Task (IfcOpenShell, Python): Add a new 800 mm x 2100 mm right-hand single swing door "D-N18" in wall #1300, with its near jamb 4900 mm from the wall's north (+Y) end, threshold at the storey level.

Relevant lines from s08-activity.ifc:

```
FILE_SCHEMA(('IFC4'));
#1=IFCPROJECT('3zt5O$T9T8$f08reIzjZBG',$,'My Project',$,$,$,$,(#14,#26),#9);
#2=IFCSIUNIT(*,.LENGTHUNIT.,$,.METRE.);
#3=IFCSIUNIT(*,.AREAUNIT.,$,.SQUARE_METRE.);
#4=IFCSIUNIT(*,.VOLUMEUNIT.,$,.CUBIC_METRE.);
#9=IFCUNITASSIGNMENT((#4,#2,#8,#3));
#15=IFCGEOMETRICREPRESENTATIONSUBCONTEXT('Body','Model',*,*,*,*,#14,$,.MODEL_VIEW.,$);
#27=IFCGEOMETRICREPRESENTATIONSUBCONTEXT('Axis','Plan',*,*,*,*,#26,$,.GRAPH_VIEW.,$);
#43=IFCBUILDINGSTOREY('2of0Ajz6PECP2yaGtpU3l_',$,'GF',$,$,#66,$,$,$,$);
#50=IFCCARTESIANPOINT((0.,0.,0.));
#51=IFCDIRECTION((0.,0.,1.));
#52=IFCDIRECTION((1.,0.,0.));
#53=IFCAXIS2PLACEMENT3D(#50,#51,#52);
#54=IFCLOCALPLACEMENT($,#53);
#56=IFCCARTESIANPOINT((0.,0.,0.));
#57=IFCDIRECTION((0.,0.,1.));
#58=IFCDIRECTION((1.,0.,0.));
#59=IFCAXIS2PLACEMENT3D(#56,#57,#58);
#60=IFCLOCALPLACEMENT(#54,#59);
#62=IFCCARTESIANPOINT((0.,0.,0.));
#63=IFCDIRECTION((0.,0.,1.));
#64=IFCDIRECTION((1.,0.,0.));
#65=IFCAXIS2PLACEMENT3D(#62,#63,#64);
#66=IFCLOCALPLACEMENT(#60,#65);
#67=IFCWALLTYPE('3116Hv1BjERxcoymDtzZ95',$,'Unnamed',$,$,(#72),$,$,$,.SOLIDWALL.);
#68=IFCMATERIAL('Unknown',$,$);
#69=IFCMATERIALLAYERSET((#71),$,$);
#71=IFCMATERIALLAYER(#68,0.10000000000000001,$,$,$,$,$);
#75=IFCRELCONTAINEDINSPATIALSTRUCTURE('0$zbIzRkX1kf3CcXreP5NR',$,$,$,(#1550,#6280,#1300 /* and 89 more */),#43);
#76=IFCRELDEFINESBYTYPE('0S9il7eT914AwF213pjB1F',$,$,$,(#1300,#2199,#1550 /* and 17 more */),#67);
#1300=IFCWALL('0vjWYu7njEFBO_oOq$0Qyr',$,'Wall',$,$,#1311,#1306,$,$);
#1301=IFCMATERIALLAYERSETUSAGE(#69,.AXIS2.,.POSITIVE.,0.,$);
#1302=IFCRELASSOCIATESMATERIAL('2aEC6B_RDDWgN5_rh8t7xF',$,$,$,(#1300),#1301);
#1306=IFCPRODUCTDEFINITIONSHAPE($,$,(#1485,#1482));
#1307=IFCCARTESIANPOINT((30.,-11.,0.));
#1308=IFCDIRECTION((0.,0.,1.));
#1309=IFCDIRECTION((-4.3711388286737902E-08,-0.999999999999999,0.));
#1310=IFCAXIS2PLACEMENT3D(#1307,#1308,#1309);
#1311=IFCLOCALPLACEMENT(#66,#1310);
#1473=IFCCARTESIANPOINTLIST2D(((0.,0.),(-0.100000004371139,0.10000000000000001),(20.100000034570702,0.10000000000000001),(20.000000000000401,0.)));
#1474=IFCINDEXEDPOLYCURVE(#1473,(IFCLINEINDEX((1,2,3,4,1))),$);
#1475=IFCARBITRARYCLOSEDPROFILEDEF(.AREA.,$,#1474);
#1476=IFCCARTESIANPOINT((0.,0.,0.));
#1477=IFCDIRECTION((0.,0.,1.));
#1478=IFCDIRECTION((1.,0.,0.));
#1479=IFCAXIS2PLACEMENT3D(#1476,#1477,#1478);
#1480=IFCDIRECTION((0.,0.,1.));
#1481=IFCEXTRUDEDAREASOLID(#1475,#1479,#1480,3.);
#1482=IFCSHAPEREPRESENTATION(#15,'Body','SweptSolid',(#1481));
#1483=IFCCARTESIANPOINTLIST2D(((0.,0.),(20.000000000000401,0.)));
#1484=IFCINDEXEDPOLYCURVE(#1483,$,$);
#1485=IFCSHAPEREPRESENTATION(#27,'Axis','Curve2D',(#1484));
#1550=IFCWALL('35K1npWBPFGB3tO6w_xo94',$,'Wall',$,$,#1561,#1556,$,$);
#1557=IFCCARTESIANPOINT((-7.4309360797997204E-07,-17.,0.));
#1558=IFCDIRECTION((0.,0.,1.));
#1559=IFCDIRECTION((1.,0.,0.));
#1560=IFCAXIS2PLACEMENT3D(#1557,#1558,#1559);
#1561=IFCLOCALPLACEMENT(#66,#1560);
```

```python
import numpy as np
import ifcopenshell
import ifcopenshell.api.feature
import ifcopenshell.api.geometry
import ifcopenshell.api.root
import ifcopenshell.api.spatial
import ifcopenshell.geom
import ifcopenshell.util.element
import ifcopenshell.util.placement
import ifcopenshell.util.representation
import ifcopenshell.util.shape
import ifcopenshell.util.unit

model = ifcopenshell.open("s08-activity.ifc")
unit_scale = ifcopenshell.util.unit.calculate_unit_scale(model)
settings = ifcopenshell.geom.settings()


def volume(element):
    """Net volume in cubic metres, openings subtracted."""
    shape = ifcopenshell.geom.create_shape(settings, element)
    return ifcopenshell.util.shape.get_volume(shape.geometry)


wall = model.by_guid("0vjWYu7njEFBO_oOq$0Qyr")
storey = ifcopenshell.util.element.get_container(wall, ifc_class="IfcBuildingStorey")
context = ifcopenshell.util.representation.get_context(model, "Model", "Body", "MODEL_VIEW")
before = volume(wall)

width, height, from_end, sill = 0.8, 2.1, 4.9, 0.0  # metres

# The wall runs along its own X axis, and the end named is its -X end.
wall_shape = ifcopenshell.geom.create_shape(settings, wall)
x, y, z = ifcopenshell.util.shape.get_vertices(wall_shape.geometry).T
start = x.min() + from_end
face, thickness = float(y.min()), float(y.max() - y.min())
wall_matrix = ifcopenshell.util.placement.get_local_placement(wall.ObjectPlacement)
level = ifcopenshell.util.placement.get_local_placement(storey.ObjectPlacement)[2, 3]


def in_wall(x, y):
    """Placement at x, y metres in the wall's axes, at sill height."""
    matrix = wall_matrix.copy()
    matrix[:, 3] = wall_matrix @ np.array([x / unit_scale, y / unit_scale, 0.0, 1.0])
    matrix[2, 3] = level + sill / unit_scale
    return matrix


# Opening: a box that overshoots both wall faces by 50 mm.
opening = ifcopenshell.api.root.create_entity(model, ifc_class="IfcOpeningElement", predefined_type="OPENING")
box = ifcopenshell.api.geometry.add_wall_representation(
    model, context=context, length=width, height=height, thickness=thickness + 0.1
)
ifcopenshell.api.geometry.assign_representation(model, product=opening, representation=box)
ifcopenshell.api.geometry.edit_object_placement(model, product=opening, matrix=in_wall(start, face - 0.05), is_si=False)
ifcopenshell.api.feature.add_feature(model, feature=opening, element=wall)

door = ifcopenshell.api.root.create_entity(model, ifc_class="IfcDoor", name="D-N18", predefined_type="DOOR")
door.OverallWidth, door.OverallHeight = width / unit_scale, height / unit_scale
door.OperationType = "SINGLE_SWING_RIGHT"
body = ifcopenshell.api.geometry.add_door_representation(
    model,
    context=context,
    overall_width=door.OverallWidth,
    overall_height=door.OverallHeight,
    operation_type="SINGLE_SWING_RIGHT",
    lining_properties={"LiningDepth": thickness / unit_scale, "ThresholdDepth": thickness / unit_scale},
)
ifcopenshell.api.geometry.assign_representation(model, product=door, representation=body)
ifcopenshell.api.spatial.assign_container(model, products=[door], relating_structure=storey)
ifcopenshell.api.feature.add_filling(model, opening=opening, element=door)

# The lining spans the wall, so the door starts at the wall face.
ifcopenshell.api.geometry.edit_object_placement(model, product=door, matrix=in_wall(start, face), is_si=False)

after = volume(wall)

print(f"wall volume {before:.3f} -> {after:.3f} m3")

model.write("s08-activity_edited.ifc")
```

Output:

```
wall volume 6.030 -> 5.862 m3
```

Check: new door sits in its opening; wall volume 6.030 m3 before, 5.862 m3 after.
